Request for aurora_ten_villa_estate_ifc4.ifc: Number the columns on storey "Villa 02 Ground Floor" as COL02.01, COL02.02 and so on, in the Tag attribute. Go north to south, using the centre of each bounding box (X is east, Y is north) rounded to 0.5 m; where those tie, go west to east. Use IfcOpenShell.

First a look at what the model holds.

```python
import ifcopenshell
import ifcopenshell.util.element
import ifcopenshell.util.placement

model = ifcopenshell.open("aurora_ten_villa_estate_ifc4.ifc")
print(model.schema)
storey = next(s for s in model.by_type("IfcBuildingStorey") if s.Name == "Villa 02 Ground Floor")
columns = [e for e in ifcopenshell.util.element.get_decomposition(storey) if e.is_a("IfcColumn")]
for e in sorted(columns, key=lambda e: e.id()):
    origin = ifcopenshell.util.placement.get_local_placement(e.ObjectPlacement)[:3, 3]
    print(e.id(), e.Tag, e.Name, origin.round(2) + 0.0, sep=" | ")
```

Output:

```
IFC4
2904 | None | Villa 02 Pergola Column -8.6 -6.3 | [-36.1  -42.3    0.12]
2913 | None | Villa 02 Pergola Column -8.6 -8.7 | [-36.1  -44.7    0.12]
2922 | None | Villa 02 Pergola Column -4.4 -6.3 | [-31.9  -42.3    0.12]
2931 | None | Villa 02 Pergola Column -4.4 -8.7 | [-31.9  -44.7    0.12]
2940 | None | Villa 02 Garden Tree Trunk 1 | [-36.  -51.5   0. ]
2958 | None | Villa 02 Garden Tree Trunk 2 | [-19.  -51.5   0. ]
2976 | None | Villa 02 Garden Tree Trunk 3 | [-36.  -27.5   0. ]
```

```python
import ifcopenshell
import ifcopenshell.geom
import ifcopenshell.util.element
import ifcopenshell.util.shape

model = ifcopenshell.open("aurora_ten_villa_estate_ifc4.ifc")
settings = ifcopenshell.geom.settings()
settings.set("use-world-coords", True)


def centre(element):
    shape = ifcopenshell.geom.create_shape(settings, element)
    return ifcopenshell.util.shape.get_bbox_centroid(shape.geometry)


storey = next(s for s in model.by_type("IfcBuildingStorey") if s.Name == "Villa 02 Ground Floor")
columns = [e for e in ifcopenshell.util.element.get_decomposition(storey) if e.is_a("IfcColumn")]

# Insertion points can sit at a corner or the storey origin, so sort by the geometry (in metres).
centres = {e: centre(e) for e in columns}
columns.sort(key=lambda e: (-round(centres[e][1] / 0.5), centres[e][0]))

for i, e in enumerate(columns, start=1):
    number = f"COL02.{i:02d}"
    e.Tag = number
    print(e.id(), number)

model.write("aurora_ten_villa_estate_ifc4_edited.ifc")
```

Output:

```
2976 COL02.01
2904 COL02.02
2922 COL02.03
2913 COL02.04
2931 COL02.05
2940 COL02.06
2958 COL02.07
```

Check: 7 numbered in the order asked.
